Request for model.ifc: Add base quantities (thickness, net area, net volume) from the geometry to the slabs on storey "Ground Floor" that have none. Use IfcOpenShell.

First a look at what the model holds.

```python
import ifcopenshell
import ifcopenshell.util.element
import ifcopenshell.util.unit

model = ifcopenshell.open("model.ifc")
print(model.schema)
for unit_type in ("LENGTHUNIT", "AREAUNIT", "VOLUMEUNIT"):
    print(unit_type, ifcopenshell.util.unit.calculate_unit_scale(model, unit_type))
storey = next(s for s in model.by_type("IfcBuildingStorey") if s.Name == "Ground Floor")
slabs = [e for e in ifcopenshell.util.element.get_decomposition(storey) if e.is_a("IfcSlab")]
for e in sorted(slabs, key=lambda e: e.id()):
    print(e.id(), e.is_a(), e.Name, list(ifcopenshell.util.element.get_psets(e, qtos_only=True)), sep=" | ")
```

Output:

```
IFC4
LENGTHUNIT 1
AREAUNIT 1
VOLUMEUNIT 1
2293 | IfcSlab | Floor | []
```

```python
import ifcopenshell
import ifcopenshell.api.pset
import ifcopenshell.geom
import ifcopenshell.util.element
import ifcopenshell.util.shape
import ifcopenshell.util.unit

model = ifcopenshell.open("model.ifc")
unit_scale = ifcopenshell.util.unit.calculate_unit_scale(model)
area_scale = ifcopenshell.util.unit.calculate_unit_scale(model, "AREAUNIT")
volume_scale = ifcopenshell.util.unit.calculate_unit_scale(model, "VOLUMEUNIT")
settings = ifcopenshell.geom.settings()

storey = next(s for s in model.by_type("IfcBuildingStorey") if s.Name == "Ground Floor")
slabs = [e for e in ifcopenshell.util.element.get_decomposition(storey) if e.is_a("IfcSlab")]

for e in sorted(slabs, key=lambda e: e.id()):
    if ifcopenshell.util.element.get_psets(e, qtos_only=True, should_inherit=False):
        continue
    # Geometry comes back in metres, in the element's own axes.
    shape = ifcopenshell.geom.create_shape(settings, e)
    values = {
        "Width": ifcopenshell.util.shape.get_z(shape.geometry) / unit_scale,
        "NetArea": ifcopenshell.util.shape.get_footprint_area(shape.geometry) / area_scale,
        "NetVolume": ifcopenshell.util.shape.get_volume(shape.geometry) / volume_scale,
    }
    qto = ifcopenshell.api.pset.add_qto(model, product=e, name="Qto_SlabBaseQuantities")
    ifcopenshell.api.pset.edit_qto(model, qto=qto, properties=values)
    print(e.id(), {k: round(v, 3) for k, v in values.items()})

model.write("model_v2.ifc")
```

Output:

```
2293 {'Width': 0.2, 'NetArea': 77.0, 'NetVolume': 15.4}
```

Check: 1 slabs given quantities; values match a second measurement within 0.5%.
